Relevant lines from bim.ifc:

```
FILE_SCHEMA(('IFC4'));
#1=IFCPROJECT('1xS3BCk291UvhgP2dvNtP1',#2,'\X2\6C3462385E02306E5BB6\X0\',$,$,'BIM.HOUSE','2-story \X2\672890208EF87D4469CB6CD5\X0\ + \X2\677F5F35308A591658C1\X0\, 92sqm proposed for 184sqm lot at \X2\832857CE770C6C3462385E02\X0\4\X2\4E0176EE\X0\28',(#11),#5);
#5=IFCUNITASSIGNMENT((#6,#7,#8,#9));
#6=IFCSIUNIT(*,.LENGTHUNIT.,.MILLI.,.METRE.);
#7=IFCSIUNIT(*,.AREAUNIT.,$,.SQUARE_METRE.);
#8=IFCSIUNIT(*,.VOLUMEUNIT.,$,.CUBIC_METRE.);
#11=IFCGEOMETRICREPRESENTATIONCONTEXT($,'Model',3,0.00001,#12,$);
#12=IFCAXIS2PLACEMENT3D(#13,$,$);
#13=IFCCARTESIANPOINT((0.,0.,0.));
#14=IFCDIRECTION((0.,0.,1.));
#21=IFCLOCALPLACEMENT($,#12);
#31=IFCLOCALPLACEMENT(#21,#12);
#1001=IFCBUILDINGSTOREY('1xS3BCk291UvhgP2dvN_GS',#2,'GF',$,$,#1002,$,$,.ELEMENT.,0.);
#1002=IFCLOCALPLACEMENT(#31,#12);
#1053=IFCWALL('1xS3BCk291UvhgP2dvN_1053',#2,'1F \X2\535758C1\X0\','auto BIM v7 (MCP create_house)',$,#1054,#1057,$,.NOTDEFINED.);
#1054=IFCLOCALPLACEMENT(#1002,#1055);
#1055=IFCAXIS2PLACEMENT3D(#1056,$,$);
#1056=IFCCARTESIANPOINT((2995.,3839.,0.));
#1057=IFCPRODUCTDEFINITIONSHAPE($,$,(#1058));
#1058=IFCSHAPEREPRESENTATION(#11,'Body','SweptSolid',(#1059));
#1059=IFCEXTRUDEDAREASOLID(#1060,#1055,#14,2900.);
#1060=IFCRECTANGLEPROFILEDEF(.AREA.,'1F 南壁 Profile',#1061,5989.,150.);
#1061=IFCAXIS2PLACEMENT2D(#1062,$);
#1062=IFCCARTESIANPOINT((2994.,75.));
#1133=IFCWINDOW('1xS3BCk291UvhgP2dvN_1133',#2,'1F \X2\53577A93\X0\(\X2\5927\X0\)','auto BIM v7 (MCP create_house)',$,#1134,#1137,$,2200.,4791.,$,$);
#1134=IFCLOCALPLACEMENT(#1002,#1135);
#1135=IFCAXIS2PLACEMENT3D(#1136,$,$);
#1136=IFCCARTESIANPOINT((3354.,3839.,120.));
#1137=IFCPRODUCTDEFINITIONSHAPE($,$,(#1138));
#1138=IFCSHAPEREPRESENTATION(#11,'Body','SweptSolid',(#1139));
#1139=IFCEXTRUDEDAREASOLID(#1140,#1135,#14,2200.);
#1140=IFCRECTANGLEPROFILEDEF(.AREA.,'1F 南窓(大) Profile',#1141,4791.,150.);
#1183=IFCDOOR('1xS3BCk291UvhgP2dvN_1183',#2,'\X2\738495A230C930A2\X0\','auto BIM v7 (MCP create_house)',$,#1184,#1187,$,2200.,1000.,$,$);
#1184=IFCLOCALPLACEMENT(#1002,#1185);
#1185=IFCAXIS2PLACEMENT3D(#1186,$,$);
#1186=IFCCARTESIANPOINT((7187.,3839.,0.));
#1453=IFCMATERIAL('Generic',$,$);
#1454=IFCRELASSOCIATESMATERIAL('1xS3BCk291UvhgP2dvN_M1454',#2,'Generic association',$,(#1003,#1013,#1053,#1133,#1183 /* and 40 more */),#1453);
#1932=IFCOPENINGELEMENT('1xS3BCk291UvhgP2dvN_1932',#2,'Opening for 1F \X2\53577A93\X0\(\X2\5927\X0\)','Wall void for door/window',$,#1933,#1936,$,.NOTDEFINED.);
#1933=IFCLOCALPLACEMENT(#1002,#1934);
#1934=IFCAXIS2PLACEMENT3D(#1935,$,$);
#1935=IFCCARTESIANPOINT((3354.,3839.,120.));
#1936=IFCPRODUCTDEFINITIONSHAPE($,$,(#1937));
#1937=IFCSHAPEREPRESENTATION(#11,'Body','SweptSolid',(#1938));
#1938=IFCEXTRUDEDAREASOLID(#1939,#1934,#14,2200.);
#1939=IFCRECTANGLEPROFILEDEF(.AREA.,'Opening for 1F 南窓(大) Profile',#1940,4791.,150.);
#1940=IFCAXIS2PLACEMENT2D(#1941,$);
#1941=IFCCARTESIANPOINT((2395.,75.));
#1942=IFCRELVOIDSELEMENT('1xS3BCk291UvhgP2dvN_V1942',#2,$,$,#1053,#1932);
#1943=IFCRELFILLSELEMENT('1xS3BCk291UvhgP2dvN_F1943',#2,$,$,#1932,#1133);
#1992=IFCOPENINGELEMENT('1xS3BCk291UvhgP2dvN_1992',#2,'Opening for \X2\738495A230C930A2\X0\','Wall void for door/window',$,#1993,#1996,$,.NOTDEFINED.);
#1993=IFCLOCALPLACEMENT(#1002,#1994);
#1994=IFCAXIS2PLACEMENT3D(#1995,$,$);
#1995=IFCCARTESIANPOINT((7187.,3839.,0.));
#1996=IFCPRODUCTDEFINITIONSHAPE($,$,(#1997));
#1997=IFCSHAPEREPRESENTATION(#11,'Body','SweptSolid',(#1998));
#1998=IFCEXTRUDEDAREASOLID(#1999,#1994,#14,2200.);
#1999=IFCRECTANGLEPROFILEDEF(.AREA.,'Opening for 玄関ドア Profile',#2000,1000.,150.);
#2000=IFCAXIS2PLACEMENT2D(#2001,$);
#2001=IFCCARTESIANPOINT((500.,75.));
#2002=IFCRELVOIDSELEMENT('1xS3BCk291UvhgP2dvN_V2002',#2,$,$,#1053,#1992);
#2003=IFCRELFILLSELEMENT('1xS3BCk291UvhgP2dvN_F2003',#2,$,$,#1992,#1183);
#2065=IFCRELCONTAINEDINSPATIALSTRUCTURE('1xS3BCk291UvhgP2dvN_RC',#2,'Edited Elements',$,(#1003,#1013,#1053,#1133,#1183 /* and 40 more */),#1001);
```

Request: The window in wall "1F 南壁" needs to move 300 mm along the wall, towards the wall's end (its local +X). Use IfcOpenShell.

```python
import ifcopenshell
import ifcopenshell.api.geometry
import ifcopenshell.util.placement
import ifcopenshell.util.unit

model = ifcopenshell.open("bim.ifc")
unit_scale = ifcopenshell.util.unit.calculate_unit_scale(model)

window = model.by_guid("1xS3BCk291UvhgP2dvN_1133")
opening = window.FillsVoids[0].RelatingOpeningElement
wall = opening.VoidsElements[0].RelatingBuildingElement

wall_matrix = ifcopenshell.util.placement.get_local_placement(wall.ObjectPlacement)
shift = wall_matrix[:3, 0] * 0.3 / unit_scale
before = ifcopenshell.util.placement.get_local_placement(window.ObjectPlacement)[:3, 3].copy()

# The window is not placed relative to its opening, so move both.
for product in (opening, window):
    matrix = ifcopenshell.util.placement.get_local_placement(product.ObjectPlacement)
    matrix[:3, 3] += shift
    ifcopenshell.api.geometry.edit_object_placement(model, product=product, matrix=matrix, is_si=False)

after = ifcopenshell.util.placement.get_local_placement(window.ObjectPlacement)[:3, 3]
print("window moved by", (after - before).round(3) + 0.0)

model.write("bim_edited.ifc")
```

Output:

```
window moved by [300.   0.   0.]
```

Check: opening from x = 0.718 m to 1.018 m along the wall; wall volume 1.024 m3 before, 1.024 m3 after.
